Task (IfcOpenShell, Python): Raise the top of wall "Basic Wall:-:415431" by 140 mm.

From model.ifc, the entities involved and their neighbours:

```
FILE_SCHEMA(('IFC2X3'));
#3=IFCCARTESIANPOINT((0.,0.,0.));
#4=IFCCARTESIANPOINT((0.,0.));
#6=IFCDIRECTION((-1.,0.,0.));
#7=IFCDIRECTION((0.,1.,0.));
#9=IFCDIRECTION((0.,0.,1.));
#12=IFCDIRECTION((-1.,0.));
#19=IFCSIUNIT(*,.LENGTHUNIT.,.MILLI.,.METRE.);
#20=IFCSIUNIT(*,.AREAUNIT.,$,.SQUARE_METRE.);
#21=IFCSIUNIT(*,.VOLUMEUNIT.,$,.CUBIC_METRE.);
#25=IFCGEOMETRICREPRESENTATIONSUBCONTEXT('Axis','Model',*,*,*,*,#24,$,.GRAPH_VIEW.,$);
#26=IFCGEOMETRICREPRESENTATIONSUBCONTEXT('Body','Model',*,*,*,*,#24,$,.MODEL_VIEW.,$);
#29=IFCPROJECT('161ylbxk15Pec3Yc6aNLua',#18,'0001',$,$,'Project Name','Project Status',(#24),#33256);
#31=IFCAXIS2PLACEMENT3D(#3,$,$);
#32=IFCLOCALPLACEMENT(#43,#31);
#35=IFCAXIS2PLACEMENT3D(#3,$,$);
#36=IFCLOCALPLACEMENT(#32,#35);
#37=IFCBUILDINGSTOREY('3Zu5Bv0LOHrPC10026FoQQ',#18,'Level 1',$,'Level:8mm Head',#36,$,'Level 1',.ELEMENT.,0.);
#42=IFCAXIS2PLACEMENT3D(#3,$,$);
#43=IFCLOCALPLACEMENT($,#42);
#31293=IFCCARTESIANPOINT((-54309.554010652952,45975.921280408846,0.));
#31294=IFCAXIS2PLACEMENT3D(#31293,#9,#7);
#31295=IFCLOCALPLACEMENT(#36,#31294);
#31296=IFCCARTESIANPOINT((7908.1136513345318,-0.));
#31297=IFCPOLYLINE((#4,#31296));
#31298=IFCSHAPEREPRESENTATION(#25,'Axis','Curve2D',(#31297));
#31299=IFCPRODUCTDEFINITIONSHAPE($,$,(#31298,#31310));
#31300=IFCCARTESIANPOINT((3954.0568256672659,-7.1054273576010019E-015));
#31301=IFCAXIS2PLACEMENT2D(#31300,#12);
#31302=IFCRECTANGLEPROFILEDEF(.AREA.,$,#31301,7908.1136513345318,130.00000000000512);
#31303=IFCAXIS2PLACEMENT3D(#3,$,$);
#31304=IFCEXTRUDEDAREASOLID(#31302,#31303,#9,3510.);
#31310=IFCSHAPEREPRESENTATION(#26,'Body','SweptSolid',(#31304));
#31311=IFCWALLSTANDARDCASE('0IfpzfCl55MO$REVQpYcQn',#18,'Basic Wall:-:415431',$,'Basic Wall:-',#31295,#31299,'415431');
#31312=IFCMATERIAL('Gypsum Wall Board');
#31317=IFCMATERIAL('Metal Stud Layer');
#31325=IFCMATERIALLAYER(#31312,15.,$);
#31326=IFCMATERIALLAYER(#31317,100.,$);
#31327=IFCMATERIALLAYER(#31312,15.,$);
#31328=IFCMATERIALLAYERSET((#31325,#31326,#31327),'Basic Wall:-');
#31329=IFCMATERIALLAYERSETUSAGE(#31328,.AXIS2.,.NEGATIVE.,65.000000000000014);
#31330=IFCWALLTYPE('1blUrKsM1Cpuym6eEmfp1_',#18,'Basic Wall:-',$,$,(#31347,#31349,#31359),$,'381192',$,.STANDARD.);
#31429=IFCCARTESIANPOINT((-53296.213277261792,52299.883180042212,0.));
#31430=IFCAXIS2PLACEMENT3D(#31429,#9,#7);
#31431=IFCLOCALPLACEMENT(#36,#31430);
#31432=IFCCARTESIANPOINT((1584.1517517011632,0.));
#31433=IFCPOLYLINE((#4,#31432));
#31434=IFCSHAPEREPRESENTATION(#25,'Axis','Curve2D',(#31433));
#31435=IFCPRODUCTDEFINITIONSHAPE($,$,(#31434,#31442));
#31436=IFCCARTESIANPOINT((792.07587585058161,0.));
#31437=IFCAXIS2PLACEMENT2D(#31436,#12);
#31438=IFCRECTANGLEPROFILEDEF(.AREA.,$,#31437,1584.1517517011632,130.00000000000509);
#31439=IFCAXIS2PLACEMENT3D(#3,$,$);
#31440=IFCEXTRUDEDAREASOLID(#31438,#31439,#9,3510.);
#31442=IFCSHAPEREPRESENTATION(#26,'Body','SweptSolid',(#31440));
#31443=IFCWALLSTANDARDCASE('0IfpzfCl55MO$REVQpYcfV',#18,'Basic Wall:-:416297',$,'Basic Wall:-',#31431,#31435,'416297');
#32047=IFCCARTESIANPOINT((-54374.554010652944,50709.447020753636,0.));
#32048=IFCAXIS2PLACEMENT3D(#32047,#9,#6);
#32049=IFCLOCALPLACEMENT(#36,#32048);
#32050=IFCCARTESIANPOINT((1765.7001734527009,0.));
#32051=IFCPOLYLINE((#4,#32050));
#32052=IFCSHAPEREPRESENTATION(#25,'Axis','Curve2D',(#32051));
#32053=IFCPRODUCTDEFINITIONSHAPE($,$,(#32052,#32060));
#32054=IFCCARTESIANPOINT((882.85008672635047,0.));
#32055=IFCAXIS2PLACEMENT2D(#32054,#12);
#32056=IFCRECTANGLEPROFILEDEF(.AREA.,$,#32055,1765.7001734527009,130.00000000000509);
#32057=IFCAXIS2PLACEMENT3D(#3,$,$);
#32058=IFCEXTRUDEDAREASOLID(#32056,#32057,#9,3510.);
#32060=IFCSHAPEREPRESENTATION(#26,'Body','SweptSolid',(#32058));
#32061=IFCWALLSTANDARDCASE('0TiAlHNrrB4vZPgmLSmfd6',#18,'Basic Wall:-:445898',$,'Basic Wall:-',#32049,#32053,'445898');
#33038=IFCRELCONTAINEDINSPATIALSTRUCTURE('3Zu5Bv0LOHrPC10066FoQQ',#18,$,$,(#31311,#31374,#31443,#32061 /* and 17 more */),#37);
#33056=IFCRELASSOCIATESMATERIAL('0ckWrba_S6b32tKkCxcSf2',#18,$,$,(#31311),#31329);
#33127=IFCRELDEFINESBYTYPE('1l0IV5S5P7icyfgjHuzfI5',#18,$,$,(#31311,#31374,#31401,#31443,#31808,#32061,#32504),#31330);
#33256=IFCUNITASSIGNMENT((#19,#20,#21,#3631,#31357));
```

```python
import ifcopenshell
import ifcopenshell.geom
import ifcopenshell.util.representation
import ifcopenshell.util.shape
import ifcopenshell.util.unit

model = ifcopenshell.open("model.ifc")
unit_scale = ifcopenshell.util.unit.calculate_unit_scale(model)
settings = ifcopenshell.geom.settings()


def volume(element):
    """Net volume in cubic metres, openings subtracted."""
    shape = ifcopenshell.geom.create_shape(settings, element)
    return ifcopenshell.util.shape.get_volume(shape.geometry)


wall = model.by_guid("0IfpzfCl55MO$REVQpYcQn")
before = volume(wall)

body = ifcopenshell.util.representation.get_representation(wall, "Model", "Body")
solid = body.Items[0]
old_height = solid.Depth
solid.Depth += 0.14 / unit_scale
after = volume(wall)

print(f"height {old_height:g} -> {solid.Depth:g}, volume {before:.3f} -> {after:.3f} m3")

model.write("model_v2.ifc")
```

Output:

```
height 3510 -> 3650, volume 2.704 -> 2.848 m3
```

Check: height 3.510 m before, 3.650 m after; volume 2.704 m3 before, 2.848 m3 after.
